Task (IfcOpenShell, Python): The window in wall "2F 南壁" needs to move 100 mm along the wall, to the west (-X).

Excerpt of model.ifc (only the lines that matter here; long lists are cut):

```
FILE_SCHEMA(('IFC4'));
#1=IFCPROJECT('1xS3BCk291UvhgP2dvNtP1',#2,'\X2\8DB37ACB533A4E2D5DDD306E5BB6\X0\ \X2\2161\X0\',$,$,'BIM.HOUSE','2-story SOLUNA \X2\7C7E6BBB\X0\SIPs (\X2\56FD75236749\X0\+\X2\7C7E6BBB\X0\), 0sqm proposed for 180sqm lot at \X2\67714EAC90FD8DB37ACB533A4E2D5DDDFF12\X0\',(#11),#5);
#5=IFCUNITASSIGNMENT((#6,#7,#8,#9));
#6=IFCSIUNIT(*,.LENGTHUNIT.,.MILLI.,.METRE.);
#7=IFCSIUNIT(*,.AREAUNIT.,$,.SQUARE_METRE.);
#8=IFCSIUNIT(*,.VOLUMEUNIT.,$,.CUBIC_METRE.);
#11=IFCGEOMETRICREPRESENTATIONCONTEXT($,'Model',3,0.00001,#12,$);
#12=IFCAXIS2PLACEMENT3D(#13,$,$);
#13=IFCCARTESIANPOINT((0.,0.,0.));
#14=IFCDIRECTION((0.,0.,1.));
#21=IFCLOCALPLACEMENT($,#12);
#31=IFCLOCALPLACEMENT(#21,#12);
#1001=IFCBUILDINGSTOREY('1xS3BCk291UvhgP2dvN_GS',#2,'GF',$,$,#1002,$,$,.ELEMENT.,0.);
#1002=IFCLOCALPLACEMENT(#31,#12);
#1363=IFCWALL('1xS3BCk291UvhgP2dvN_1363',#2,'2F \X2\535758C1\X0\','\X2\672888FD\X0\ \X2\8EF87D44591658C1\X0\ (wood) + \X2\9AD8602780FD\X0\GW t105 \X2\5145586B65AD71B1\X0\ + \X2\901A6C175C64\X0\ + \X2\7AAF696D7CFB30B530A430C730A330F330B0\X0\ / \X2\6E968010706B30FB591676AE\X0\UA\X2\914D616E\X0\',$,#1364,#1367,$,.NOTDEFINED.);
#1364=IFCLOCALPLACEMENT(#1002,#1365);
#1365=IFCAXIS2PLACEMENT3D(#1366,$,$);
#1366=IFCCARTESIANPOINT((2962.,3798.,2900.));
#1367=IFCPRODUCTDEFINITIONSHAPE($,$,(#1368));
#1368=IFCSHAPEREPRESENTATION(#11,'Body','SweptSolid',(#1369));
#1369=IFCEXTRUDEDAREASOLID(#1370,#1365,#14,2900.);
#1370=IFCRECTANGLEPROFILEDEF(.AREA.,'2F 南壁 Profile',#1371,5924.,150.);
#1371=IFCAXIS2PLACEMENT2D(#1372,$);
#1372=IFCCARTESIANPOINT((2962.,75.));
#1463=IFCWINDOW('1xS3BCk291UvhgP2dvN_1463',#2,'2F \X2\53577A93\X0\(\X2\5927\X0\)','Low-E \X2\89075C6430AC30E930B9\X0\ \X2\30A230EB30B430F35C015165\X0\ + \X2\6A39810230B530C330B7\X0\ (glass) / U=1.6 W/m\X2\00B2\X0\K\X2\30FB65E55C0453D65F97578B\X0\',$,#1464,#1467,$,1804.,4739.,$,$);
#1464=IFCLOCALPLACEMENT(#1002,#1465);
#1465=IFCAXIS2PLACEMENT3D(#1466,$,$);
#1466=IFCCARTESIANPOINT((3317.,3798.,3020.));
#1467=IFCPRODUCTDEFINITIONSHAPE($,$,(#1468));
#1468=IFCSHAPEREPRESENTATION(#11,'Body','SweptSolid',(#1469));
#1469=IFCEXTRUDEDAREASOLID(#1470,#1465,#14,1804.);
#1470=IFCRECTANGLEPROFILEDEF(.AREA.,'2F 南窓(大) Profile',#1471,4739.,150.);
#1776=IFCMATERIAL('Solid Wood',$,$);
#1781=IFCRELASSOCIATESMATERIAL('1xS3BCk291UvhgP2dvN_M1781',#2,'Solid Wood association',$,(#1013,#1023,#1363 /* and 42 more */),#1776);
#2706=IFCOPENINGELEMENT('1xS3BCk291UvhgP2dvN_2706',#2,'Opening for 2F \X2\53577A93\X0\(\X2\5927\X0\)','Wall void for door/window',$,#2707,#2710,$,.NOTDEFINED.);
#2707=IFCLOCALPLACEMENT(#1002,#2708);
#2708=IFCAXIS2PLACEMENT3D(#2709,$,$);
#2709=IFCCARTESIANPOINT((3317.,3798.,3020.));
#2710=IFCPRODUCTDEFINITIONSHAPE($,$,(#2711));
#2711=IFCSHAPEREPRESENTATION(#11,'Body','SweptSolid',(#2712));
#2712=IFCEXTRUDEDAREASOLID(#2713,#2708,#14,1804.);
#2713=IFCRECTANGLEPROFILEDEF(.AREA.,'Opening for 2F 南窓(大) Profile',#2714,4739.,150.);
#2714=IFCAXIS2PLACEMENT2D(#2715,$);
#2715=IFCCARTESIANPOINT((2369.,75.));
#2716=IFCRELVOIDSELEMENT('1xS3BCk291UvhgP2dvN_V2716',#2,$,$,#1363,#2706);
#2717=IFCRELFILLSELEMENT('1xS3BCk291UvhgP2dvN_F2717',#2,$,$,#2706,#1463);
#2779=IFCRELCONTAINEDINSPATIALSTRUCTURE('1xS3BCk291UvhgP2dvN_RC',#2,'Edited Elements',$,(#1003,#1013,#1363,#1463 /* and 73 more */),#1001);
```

```python
import ifcopenshell
import ifcopenshell.api.geometry
import ifcopenshell.util.placement
import ifcopenshell.util.unit

model = ifcopenshell.open("model.ifc")
unit_scale = ifcopenshell.util.unit.calculate_unit_scale(model)

window = model.by_guid("1xS3BCk291UvhgP2dvN_1463")
opening = window.FillsVoids[0].RelatingOpeningElement
wall = opening.VoidsElements[0].RelatingBuildingElement

wall_matrix = ifcopenshell.util.placement.get_local_placement(wall.ObjectPlacement)
shift = wall_matrix[:3, 0] * -0.1 / unit_scale
before = ifcopenshell.util.placement.get_local_placement(window.ObjectPlacement)[:3, 3].copy()

# The window is not placed relative to its opening, so move both.
for product in (opening, window):
    matrix = ifcopenshell.util.placement.get_local_placement(product.ObjectPlacement)
    matrix[:3, 3] += shift
    ifcopenshell.api.geometry.edit_object_placement(model, product=product, matrix=matrix, is_si=False)

after = ifcopenshell.util.placement.get_local_placement(window.ObjectPlacement)[:3, 3]
print("window moved by", (after - before).round(3) + 0.0)

model.write("model_rev.ifc")
```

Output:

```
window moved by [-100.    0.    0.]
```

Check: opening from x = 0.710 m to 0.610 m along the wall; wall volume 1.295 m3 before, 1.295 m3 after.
